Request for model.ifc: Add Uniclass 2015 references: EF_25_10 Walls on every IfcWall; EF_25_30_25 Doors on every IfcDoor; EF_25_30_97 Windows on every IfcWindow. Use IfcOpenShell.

First a look at what the model holds.

```python
import ifcopenshell

model = ifcopenshell.open("model.ifc")
print(model.schema)
print("classifications:", [c.Name for c in model.by_type("IfcClassification")])
for ifc_class in ("IfcDoor", "IfcRoof", "IfcStair", "IfcWall", "IfcWindow"):
    print(ifc_class, len(model.by_type(ifc_class)))
```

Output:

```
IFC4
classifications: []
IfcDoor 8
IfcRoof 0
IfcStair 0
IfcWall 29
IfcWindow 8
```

```python
import ifcopenshell
import ifcopenshell.api.classification

model = ifcopenshell.open("model.ifc")

system = ifcopenshell.api.classification.add_classification(model, classification="Uniclass 2015")

codes = {
    "IfcWall": ("EF_25_10", "Walls"),
    "IfcDoor": ("EF_25_30_25", "Doors"),
    "IfcWindow": ("EF_25_30_97", "Windows"),
}
for ifc_class, (code, name) in codes.items():
    products = model.by_type(ifc_class)
    ifcopenshell.api.classification.add_reference(
        model, products=products, classification=system, identification=code, name=name
    )
    print(code, len(products))

model.write("model_updated.ifc")
```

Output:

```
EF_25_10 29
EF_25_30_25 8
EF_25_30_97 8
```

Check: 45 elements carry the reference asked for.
